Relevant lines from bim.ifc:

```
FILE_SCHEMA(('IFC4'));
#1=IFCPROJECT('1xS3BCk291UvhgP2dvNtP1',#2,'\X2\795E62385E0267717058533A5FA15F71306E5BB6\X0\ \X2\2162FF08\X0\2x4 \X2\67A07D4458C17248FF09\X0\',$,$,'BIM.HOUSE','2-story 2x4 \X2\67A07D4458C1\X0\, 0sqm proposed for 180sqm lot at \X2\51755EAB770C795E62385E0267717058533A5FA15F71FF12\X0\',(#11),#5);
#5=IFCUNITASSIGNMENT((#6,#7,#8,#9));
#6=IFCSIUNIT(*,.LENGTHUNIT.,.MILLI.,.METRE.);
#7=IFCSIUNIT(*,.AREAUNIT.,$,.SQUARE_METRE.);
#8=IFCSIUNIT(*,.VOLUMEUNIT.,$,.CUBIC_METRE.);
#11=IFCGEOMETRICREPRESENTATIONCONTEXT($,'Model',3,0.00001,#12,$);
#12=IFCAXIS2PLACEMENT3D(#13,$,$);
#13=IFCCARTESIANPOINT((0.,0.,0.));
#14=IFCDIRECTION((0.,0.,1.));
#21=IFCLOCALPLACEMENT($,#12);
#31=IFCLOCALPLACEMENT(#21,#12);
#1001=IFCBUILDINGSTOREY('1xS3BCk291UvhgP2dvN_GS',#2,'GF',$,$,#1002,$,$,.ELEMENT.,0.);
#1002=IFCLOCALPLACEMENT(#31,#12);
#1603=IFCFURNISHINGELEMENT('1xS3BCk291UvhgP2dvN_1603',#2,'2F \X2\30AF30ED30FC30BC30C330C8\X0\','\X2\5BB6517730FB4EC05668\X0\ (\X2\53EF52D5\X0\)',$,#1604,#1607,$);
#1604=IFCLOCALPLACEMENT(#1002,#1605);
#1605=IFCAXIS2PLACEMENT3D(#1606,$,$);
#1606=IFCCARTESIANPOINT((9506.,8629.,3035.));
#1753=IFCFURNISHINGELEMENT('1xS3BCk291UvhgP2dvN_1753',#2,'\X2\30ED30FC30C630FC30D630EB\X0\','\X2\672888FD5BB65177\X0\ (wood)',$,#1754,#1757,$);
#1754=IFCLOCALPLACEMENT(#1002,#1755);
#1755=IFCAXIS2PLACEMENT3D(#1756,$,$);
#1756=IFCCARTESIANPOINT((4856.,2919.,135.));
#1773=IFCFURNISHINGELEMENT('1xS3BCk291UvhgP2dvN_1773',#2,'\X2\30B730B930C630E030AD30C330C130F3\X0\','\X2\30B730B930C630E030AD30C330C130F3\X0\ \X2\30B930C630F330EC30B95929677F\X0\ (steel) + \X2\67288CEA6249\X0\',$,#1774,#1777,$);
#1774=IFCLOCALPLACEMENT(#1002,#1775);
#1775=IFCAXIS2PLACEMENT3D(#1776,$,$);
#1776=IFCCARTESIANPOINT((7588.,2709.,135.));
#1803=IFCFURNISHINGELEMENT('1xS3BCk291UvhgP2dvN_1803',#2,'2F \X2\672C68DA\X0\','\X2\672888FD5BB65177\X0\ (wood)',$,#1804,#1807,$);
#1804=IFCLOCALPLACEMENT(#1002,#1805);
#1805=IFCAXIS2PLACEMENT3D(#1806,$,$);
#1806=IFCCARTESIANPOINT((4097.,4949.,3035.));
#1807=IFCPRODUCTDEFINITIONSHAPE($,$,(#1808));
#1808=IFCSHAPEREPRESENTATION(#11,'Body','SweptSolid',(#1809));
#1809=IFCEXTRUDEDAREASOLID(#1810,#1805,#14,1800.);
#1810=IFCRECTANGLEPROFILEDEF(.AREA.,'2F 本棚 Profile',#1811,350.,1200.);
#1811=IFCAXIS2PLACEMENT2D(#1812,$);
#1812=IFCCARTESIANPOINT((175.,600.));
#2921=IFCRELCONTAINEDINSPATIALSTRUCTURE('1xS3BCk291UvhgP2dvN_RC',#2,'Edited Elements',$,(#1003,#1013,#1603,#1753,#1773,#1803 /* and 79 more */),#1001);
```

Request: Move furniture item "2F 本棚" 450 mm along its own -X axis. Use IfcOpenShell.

```python
import ifcopenshell
import ifcopenshell.api.geometry
import ifcopenshell.util.placement
import ifcopenshell.util.unit

model = ifcopenshell.open("bim.ifc")
unit_scale = ifcopenshell.util.unit.calculate_unit_scale(model)

item = model.by_guid("1xS3BCk291UvhgP2dvN_1803")
matrix = ifcopenshell.util.placement.get_local_placement(item.ObjectPlacement)
matrix[:3, 3] -= matrix[:3, 0] * 0.45 / unit_scale
ifcopenshell.api.geometry.edit_object_placement(model, product=item, matrix=matrix, is_si=False)

print(ifcopenshell.util.placement.get_local_placement(item.ObjectPlacement).round(3) + 0.0)

model.write("bim_v2.ifc")
```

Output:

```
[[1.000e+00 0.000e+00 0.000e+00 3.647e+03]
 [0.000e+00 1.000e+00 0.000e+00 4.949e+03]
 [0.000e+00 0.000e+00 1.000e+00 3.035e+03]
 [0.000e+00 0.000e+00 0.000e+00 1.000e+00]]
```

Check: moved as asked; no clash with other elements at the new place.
